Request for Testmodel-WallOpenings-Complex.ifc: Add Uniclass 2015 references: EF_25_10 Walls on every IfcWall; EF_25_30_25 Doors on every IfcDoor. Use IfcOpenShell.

First a look at what the model holds.

```python
import ifcopenshell

model = ifcopenshell.open("Testmodel-WallOpenings-Complex.ifc")
print(model.schema)
print("classifications:", [c.Name for c in model.by_type("IfcClassification")])
for ifc_class in ("IfcDoor", "IfcRoof", "IfcStair", "IfcWall", "IfcWindow"):
    print(ifc_class, len(model.by_type(ifc_class)))
```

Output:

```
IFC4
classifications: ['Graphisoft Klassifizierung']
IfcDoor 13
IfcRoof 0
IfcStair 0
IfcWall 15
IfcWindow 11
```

```python
import ifcopenshell
import ifcopenshell.api.classification

model = ifcopenshell.open("Testmodel-WallOpenings-Complex.ifc")

system = ifcopenshell.api.classification.add_classification(model, classification="Uniclass 2015")

codes = {
    "IfcWall": ("EF_25_10", "Walls"),
    "IfcDoor": ("EF_25_30_25", "Doors"),
}
for ifc_class, (code, name) in codes.items():
    products = model.by_type(ifc_class)
    ifcopenshell.api.classification.add_reference(
        model, products=products, classification=system, identification=code, name=name
    )
    print(code, len(products))

model.write("Testmodel-WallOpenings-Complex_updated.ifc")
```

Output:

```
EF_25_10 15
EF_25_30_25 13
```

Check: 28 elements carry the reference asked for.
